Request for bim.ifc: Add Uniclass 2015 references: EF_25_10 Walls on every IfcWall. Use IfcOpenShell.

First a look at what the model holds.

```python
import ifcopenshell

model = ifcopenshell.open("bim.ifc")
print(model.schema)
print("classifications:", [c.Name for c in model.by_type("IfcClassification")])
for ifc_class in ("IfcDoor", "IfcRoof", "IfcStair", "IfcWall", "IfcWindow"):
    print(ifc_class, len(model.by_type(ifc_class)))
```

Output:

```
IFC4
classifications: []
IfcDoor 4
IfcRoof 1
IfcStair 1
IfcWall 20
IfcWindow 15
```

```python
import ifcopenshell
import ifcopenshell.api.classification

model = ifcopenshell.open("bim.ifc")

system = ifcopenshell.api.classification.add_classification(model, classification="Uniclass 2015")

codes = {
    "IfcWall": ("EF_25_10", "Walls"),
}
for ifc_class, (code, name) in codes.items():
    products = model.by_type(ifc_class)
    ifcopenshell.api.classification.add_reference(
        model, products=products, classification=system, identification=code, name=name
    )
    print(code, len(products))

model.write("bim_edited.ifc")
```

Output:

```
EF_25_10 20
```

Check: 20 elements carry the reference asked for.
